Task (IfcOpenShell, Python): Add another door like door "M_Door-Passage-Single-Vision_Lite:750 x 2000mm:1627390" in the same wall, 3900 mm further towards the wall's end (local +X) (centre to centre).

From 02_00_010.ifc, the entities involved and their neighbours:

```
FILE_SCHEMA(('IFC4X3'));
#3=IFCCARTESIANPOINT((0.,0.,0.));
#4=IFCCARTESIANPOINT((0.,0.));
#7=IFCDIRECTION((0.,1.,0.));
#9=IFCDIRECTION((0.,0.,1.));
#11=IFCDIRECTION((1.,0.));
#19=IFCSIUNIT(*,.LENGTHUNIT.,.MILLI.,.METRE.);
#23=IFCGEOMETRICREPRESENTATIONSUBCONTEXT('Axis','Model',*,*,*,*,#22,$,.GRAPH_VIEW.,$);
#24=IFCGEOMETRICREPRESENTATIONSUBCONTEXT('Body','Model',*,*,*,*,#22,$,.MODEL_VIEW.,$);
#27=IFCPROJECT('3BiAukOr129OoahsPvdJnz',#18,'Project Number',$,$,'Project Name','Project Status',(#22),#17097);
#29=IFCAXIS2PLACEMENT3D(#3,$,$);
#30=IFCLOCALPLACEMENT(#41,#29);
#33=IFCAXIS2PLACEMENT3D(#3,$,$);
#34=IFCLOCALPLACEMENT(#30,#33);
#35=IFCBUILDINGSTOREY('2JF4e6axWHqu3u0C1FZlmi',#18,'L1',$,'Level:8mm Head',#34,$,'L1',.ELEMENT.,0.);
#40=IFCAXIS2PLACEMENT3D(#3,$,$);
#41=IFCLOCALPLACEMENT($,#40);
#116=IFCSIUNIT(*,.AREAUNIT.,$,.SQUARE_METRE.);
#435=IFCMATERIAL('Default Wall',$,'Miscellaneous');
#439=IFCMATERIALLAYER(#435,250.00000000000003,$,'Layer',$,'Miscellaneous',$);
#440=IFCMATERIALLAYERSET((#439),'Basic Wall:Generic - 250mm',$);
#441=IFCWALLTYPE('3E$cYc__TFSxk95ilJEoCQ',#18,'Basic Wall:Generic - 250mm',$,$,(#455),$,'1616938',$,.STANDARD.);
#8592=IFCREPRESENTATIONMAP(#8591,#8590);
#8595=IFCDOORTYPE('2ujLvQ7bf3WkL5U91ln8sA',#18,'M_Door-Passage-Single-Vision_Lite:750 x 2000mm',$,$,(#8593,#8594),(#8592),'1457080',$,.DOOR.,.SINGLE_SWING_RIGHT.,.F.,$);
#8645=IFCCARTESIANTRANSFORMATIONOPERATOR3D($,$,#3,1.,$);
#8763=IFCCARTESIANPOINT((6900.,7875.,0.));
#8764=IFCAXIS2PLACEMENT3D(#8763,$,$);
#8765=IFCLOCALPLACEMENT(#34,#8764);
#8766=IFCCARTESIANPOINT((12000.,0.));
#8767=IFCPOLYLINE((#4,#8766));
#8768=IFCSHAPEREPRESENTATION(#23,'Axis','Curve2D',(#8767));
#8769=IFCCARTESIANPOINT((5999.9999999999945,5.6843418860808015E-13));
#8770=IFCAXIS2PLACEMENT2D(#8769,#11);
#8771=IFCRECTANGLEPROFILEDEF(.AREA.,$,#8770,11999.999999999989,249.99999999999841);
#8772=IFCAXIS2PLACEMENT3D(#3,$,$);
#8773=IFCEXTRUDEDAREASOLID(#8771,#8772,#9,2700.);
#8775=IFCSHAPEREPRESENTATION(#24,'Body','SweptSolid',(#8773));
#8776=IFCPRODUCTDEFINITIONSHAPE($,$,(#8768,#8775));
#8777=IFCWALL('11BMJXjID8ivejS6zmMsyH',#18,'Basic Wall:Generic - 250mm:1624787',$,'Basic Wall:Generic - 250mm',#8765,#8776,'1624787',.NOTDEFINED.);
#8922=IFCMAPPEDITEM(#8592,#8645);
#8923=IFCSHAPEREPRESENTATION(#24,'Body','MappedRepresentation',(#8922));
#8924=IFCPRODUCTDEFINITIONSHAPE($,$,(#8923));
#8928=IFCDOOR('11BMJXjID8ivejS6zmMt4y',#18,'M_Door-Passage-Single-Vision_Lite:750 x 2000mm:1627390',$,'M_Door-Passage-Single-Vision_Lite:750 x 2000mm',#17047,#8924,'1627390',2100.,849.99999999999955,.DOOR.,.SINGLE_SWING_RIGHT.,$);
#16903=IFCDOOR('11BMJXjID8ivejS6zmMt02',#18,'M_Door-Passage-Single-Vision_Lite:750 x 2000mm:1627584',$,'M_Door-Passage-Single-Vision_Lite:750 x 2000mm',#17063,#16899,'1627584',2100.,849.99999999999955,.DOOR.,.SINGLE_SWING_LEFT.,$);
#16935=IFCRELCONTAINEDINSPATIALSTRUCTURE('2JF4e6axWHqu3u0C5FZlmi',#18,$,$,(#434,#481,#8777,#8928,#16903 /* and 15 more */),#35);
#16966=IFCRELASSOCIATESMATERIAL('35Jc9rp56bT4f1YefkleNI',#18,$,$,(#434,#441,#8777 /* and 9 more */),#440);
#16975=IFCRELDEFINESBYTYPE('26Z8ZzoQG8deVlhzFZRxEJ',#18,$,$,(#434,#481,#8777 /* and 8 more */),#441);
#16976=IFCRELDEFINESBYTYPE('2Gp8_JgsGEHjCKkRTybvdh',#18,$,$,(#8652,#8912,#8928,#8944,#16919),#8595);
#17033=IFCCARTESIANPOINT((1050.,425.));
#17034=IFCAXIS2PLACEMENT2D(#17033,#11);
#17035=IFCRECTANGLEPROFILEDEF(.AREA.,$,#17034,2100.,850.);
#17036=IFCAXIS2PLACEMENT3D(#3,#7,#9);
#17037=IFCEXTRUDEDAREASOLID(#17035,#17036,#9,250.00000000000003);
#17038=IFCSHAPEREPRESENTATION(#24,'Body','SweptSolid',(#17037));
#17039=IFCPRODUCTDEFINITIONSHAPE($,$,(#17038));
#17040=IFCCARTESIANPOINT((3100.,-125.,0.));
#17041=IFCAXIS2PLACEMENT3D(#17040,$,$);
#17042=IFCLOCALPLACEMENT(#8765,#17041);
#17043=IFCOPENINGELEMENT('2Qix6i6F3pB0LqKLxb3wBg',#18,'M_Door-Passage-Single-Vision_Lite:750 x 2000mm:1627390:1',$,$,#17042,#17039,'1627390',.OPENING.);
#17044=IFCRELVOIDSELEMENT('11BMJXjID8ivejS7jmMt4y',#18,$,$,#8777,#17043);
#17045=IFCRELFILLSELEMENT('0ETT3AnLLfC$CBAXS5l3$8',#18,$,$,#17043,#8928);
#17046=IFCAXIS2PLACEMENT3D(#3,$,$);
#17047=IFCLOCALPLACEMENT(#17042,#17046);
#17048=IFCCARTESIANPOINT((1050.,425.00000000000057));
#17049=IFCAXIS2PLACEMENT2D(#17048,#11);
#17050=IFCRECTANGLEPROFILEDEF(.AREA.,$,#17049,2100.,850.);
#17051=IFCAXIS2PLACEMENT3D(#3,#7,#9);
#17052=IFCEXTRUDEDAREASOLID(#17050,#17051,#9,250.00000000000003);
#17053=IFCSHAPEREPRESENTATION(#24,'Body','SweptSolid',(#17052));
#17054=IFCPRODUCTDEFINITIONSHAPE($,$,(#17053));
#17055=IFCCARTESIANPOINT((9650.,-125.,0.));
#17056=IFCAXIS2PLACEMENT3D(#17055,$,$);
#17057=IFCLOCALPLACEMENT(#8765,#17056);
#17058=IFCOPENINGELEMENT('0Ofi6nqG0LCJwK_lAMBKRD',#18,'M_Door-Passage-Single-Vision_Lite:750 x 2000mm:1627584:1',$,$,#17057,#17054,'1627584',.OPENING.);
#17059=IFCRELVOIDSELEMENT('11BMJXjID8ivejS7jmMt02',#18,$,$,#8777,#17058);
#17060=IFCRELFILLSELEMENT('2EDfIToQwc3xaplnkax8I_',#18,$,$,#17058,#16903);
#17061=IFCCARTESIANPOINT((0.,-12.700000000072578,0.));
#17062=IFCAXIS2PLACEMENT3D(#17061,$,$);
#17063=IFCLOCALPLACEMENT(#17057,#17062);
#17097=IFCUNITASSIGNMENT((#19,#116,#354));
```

```python
import ifcopenshell
import ifcopenshell.api.feature
import ifcopenshell.api.geometry
import ifcopenshell.api.root
import ifcopenshell.geom
import ifcopenshell.util.element
import ifcopenshell.util.placement
import ifcopenshell.util.shape
import ifcopenshell.util.unit

model = ifcopenshell.open("02_00_010.ifc")
unit_scale = ifcopenshell.util.unit.calculate_unit_scale(model)
settings = ifcopenshell.geom.settings()


def volume(element):
    """Net volume in cubic metres, openings subtracted."""
    shape = ifcopenshell.geom.create_shape(settings, element)
    return ifcopenshell.util.shape.get_volume(shape.geometry)


def reuse_history(source, copy):
    """copy_class also copies each property set's owner history, people and application; keep the originals."""
    for rel in copy.IsDefinedBy:
        if rel.is_a("IfcRelDefinesByProperties") and (history := rel.RelatingPropertyDefinition.OwnerHistory):
            rel.RelatingPropertyDefinition.OwnerHistory = source.OwnerHistory
            ifcopenshell.util.element.remove_deep2(model, history)


door = model.by_id(8928)
opening = door.FillsVoids[0].RelatingOpeningElement
wall = opening.VoidsElements[0].RelatingBuildingElement
before = volume(wall)
shift = ifcopenshell.util.placement.get_local_placement(wall.ObjectPlacement)[:3, 0] * 3.9 / unit_scale

# copy_class copies the void relationship, type, container and properties, but no geometry.
new_opening = ifcopenshell.api.root.copy_class(model, product=opening)
new_opening.Representation = ifcopenshell.util.element.copy_deep(
    model, opening.Representation, exclude=["IfcGeometricRepresentationContext", "IfcRepresentationMap"]
)
new_opening.Name = "M_Door-Passage-Single-Vision_Lite:750 x 2000mm"
new_opening.Tag = None
new_door = ifcopenshell.api.root.copy_class(model, product=door)
new_door.Representation = ifcopenshell.util.element.copy_deep(
    model, door.Representation, exclude=["IfcGeometricRepresentationContext", "IfcRepresentationMap"]
)
new_door.Name = "M_Door-Passage-Single-Vision_Lite:750 x 2000mm"
new_door.Tag = None
reuse_history(door, new_door)
ifcopenshell.api.feature.add_filling(model, opening=new_opening, element=new_door)

for old, new in ((opening, new_opening), (door, new_door)):
    matrix = ifcopenshell.util.placement.get_local_placement(old.ObjectPlacement)
    matrix[:3, 3] += shift
    ifcopenshell.api.geometry.edit_object_placement(model, product=new, matrix=matrix, is_si=False)

after = volume(wall)

print(f"wall volume {before:.3f} -> {after:.3f} m3")

model.write("02_00_010_edited.ifc")
```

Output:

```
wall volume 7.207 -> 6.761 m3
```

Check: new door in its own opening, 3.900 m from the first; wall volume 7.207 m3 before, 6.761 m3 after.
